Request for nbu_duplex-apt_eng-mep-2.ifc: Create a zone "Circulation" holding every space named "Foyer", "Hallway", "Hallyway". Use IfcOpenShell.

First a look at what the model holds.

```python
import ifcopenshell

model = ifcopenshell.open("nbu_duplex-apt_eng-mep-2.ifc")
print(model.schema)
seen = {}
for space in model.by_type("IfcSpace"):
    seen[space.LongName] = seen.get(space.LongName, 0) + 1
for name, count in sorted(seen.items(), key=str):
    print(count, "x", name)
print("zones:", [z.Name for z in model.by_type("IfcZone")][:20])
```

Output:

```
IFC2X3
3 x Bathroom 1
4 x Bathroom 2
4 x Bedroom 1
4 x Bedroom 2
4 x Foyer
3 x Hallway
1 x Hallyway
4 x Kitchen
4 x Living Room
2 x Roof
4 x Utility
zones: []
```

```python
import ifcopenshell
import ifcopenshell.api.group
import ifcopenshell.api.root

model = ifcopenshell.open("nbu_duplex-apt_eng-mep-2.ifc")

names = {"Foyer", "Hallway", "Hallyway"}
spaces = [s for s in model.by_type("IfcSpace") if s.LongName in names]

zone = ifcopenshell.api.root.create_entity(model, ifc_class="IfcZone", name="Circulation")
ifcopenshell.api.group.assign_group(model, products=spaces, group=zone)
print(len(spaces), "spaces in", zone.Name)

model.write("nbu_duplex-apt_eng-mep-2_edited.ifc")
```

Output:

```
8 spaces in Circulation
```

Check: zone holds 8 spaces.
